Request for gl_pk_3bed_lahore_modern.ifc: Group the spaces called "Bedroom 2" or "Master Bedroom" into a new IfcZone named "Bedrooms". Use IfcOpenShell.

First a look at what the model holds.

```python
import ifcopenshell

model = ifcopenshell.open("gl_pk_3bed_lahore_modern.ifc")
print(model.schema)
seen = {}
for space in model.by_type("IfcSpace"):
    seen[space.LongName] = seen.get(space.LongName, 0) + 1
for name, count in sorted(seen.items(), key=str):
    print(count, "x", name)
print("zones:", [z.Name for z in model.by_type("IfcZone")][:20])
```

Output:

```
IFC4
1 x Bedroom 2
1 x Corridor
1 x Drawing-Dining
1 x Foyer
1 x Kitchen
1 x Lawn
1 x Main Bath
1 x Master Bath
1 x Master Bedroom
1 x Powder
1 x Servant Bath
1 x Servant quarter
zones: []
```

```python
import ifcopenshell
import ifcopenshell.api.group
import ifcopenshell.api.root

model = ifcopenshell.open("gl_pk_3bed_lahore_modern.ifc")

names = {"Bedroom 2", "Master Bedroom"}
spaces = [s for s in model.by_type("IfcSpace") if s.LongName in names]

zone = ifcopenshell.api.root.create_entity(model, ifc_class="IfcZone", name="Bedrooms")
ifcopenshell.api.group.assign_group(model, products=spaces, group=zone)
print(len(spaces), "spaces in", zone.Name)

model.write("gl_pk_3bed_lahore_modern_rev.ifc")
```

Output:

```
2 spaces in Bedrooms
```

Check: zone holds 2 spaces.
